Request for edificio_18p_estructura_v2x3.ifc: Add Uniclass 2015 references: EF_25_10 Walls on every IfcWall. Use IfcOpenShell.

First a look at what the model holds.

```python
import ifcopenshell

model = ifcopenshell.open("edificio_18p_estructura_v2x3.ifc")
print(model.schema)
print("classifications:", [c.Name for c in model.by_type("IfcClassification")])
for ifc_class in ("IfcDoor", "IfcRoof", "IfcStair", "IfcWall", "IfcWindow"):
    print(ifc_class, len(model.by_type(ifc_class)))
```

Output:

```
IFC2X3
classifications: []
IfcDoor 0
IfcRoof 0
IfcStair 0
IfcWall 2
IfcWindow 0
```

```python
import ifcopenshell
import ifcopenshell.api.classification

model = ifcopenshell.open("edificio_18p_estructura_v2x3.ifc")

# IFC2X3 requires Source and Edition and has no link from the project to the system.
system = model.create_entity("IfcClassification", Source="NBS", Edition="2015", Name="Uniclass 2015")

codes = {
    "IfcWall": ("EF_25_10", "Walls"),
}
for ifc_class, (code, name) in codes.items():
    products = model.by_type(ifc_class)
    ifcopenshell.api.classification.add_reference(
        model, products=products, classification=system, identification=code, name=name
    )
    print(code, len(products))

model.write("edificio_18p_estructura_v2x3_v2.ifc")
```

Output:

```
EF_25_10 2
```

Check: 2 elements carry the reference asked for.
